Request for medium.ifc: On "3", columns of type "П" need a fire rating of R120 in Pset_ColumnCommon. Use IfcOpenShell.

First a look at what the model holds.

```python
import ifcopenshell
import ifcopenshell.util.element

model = ifcopenshell.open("medium.ifc")
print(model.schema)
storey = next(s for s in model.by_type("IfcBuildingStorey") if s.Name == "3")
columns = [e for e in ifcopenshell.util.element.get_decomposition(storey) if e.is_a("IfcColumn")]
seen = {}
for e in columns:
    element_type = ifcopenshell.util.element.get_type(e)
    key = (element_type.Name if element_type != e and element_type else None, ifcopenshell.util.element.get_pset(e, "Pset_ColumnCommon", "FireRating"))
    seen[key] = seen.get(key, 0) + 1
for (name, value), count in sorted(seen.items(), key=str):
    print(count, "x", name, "|", value)
```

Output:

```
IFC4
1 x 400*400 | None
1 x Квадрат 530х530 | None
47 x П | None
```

```python
import ifcopenshell
import ifcopenshell.api.pset
import ifcopenshell.util.element

model = ifcopenshell.open("medium.ifc")

storey = next(s for s in model.by_type("IfcBuildingStorey") if s.Name == "3")
columns = [e for e in ifcopenshell.util.element.get_decomposition(storey) if e.is_a("IfcColumn")]

count = 0
for e in columns:
    element_type = ifcopenshell.util.element.get_type(e)
    if element_type in (None, e) or element_type.Name != "П":
        continue
    # add_pset returns the element's existing set when there is one.
    pset = ifcopenshell.api.pset.add_pset(model, product=e, name="Pset_ColumnCommon")
    ifcopenshell.api.pset.edit_pset(model, pset=pset, properties={"FireRating": "R120"})
    count += 1

print(count, "columns updated")

model.write("medium_v2.ifc")
```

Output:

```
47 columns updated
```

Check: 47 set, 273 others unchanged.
